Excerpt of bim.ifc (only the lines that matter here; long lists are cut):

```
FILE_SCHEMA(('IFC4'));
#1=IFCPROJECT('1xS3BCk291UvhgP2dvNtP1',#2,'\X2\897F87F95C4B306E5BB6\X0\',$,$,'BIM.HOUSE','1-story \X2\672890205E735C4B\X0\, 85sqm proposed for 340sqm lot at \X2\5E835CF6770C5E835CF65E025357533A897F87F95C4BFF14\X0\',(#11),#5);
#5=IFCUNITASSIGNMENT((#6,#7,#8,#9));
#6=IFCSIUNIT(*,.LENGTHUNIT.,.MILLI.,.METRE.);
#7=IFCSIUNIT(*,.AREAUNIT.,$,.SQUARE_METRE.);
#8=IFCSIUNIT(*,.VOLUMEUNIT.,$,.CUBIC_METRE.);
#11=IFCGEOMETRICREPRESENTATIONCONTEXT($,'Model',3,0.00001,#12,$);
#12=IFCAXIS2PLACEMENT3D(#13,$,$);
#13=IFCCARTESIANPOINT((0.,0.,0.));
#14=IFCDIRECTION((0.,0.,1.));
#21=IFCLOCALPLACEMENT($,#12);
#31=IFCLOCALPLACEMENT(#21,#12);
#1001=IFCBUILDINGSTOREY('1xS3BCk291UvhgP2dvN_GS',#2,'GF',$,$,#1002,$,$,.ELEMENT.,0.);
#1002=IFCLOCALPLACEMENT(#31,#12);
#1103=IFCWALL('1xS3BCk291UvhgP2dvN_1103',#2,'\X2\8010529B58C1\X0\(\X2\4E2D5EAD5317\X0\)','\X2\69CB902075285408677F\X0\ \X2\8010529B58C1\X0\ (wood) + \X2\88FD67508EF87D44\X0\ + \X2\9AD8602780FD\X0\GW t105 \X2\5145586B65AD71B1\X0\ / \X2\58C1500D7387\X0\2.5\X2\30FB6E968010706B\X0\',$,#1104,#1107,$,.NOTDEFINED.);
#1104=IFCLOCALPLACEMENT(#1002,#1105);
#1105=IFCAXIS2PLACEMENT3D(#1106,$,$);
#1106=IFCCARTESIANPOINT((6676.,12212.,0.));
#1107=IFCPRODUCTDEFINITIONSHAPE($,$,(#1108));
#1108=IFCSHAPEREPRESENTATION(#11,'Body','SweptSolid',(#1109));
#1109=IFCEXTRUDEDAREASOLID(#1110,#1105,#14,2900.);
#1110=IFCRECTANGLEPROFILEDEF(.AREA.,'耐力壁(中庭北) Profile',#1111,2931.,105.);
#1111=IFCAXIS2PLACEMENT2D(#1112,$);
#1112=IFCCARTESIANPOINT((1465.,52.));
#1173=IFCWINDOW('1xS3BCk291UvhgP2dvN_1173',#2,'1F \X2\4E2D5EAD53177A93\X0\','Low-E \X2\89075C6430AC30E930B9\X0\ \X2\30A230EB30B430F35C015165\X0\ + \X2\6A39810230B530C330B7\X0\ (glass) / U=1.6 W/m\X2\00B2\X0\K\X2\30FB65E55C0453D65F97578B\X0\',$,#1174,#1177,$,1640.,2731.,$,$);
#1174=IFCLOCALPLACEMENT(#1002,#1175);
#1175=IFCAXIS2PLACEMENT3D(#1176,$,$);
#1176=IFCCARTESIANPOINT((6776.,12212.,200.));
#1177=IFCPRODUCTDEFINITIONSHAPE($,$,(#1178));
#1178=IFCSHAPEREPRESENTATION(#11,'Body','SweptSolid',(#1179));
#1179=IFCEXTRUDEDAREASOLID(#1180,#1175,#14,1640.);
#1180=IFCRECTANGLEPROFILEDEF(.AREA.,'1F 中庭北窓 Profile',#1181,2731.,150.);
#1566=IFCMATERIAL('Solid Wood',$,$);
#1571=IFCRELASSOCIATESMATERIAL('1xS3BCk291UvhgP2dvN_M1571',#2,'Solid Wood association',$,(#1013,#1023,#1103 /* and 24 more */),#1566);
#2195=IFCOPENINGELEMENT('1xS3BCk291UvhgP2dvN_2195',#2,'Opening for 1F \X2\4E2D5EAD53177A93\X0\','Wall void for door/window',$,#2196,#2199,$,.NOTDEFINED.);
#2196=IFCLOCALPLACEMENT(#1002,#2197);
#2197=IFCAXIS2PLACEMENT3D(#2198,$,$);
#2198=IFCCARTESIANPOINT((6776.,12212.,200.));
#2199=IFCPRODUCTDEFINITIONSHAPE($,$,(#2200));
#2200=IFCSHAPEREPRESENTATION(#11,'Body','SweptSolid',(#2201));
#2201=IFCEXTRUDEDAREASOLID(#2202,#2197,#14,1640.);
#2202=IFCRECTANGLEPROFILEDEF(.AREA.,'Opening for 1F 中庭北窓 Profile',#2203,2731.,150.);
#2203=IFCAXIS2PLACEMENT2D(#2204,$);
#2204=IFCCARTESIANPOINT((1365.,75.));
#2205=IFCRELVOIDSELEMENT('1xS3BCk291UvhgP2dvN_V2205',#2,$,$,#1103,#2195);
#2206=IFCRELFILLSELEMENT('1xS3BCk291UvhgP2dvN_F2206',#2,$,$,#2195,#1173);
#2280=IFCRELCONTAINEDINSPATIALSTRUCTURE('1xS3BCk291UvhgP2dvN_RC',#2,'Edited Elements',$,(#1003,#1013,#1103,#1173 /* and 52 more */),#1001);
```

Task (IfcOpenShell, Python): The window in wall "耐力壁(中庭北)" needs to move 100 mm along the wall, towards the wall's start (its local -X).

```python
import ifcopenshell
import ifcopenshell.api.geometry
import ifcopenshell.util.placement
import ifcopenshell.util.unit

model = ifcopenshell.open("bim.ifc")
unit_scale = ifcopenshell.util.unit.calculate_unit_scale(model)

window = model.by_guid("1xS3BCk291UvhgP2dvN_1173")
opening = window.FillsVoids[0].RelatingOpeningElement
wall = opening.VoidsElements[0].RelatingBuildingElement

wall_matrix = ifcopenshell.util.placement.get_local_placement(wall.ObjectPlacement)
shift = wall_matrix[:3, 0] * -0.1 / unit_scale
before = ifcopenshell.util.placement.get_local_placement(window.ObjectPlacement)[:3, 3].copy()

# The window is not placed relative to its opening, so move both.
for product in (opening, window):
    matrix = ifcopenshell.util.placement.get_local_placement(product.ObjectPlacement)
    matrix[:3, 3] += shift
    ifcopenshell.api.geometry.edit_object_placement(model, product=product, matrix=matrix, is_si=False)

after = ifcopenshell.util.placement.get_local_placement(window.ObjectPlacement)[:3, 3]
print("window moved by", (after - before).round(3) + 0.0)

model.write("bim_v2.ifc")
```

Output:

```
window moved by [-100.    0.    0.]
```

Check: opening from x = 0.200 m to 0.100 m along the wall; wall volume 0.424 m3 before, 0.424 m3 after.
